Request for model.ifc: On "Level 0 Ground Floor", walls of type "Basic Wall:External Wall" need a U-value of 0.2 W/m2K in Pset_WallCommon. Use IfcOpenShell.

First a look at what the model holds.

```python
import ifcopenshell
import ifcopenshell.util.element

model = ifcopenshell.open("model.ifc")
print(model.schema)
storey = next(s for s in model.by_type("IfcBuildingStorey") if s.Name == "Level 0 Ground Floor")
walls = [e for e in ifcopenshell.util.element.get_decomposition(storey) if e.is_a("IfcWall")]
seen = {}
for e in walls:
    element_type = ifcopenshell.util.element.get_type(e)
    key = (element_type.Name if element_type != e and element_type else None, ifcopenshell.util.element.get_pset(e, "Pset_WallCommon", "ThermalTransmittance"))
    seen[key] = seen.get(key, 0) + 1
for (name, value), count in sorted(seen.items(), key=str):
    print(count, "x", name, "|", value)
```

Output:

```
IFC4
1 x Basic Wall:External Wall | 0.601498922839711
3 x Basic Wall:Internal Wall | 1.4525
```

```python
import ifcopenshell
import ifcopenshell.api.pset
import ifcopenshell.util.element

model = ifcopenshell.open("model.ifc")

storey = next(s for s in model.by_type("IfcBuildingStorey") if s.Name == "Level 0 Ground Floor")
walls = [e for e in ifcopenshell.util.element.get_decomposition(storey) if e.is_a("IfcWall")]

count = 0
for e in walls:
    element_type = ifcopenshell.util.element.get_type(e)
    if element_type in (None, e) or element_type.Name != "Basic Wall:External Wall":
        continue
    # add_pset returns the element's existing set when there is one.
    pset = ifcopenshell.api.pset.add_pset(model, product=e, name="Pset_WallCommon")
    ifcopenshell.api.pset.edit_pset(model, pset=pset, properties={"ThermalTransmittance": 0.2})
    count += 1

print(count, "walls updated")

model.write("model_v2.ifc")
```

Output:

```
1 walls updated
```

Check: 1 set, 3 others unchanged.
